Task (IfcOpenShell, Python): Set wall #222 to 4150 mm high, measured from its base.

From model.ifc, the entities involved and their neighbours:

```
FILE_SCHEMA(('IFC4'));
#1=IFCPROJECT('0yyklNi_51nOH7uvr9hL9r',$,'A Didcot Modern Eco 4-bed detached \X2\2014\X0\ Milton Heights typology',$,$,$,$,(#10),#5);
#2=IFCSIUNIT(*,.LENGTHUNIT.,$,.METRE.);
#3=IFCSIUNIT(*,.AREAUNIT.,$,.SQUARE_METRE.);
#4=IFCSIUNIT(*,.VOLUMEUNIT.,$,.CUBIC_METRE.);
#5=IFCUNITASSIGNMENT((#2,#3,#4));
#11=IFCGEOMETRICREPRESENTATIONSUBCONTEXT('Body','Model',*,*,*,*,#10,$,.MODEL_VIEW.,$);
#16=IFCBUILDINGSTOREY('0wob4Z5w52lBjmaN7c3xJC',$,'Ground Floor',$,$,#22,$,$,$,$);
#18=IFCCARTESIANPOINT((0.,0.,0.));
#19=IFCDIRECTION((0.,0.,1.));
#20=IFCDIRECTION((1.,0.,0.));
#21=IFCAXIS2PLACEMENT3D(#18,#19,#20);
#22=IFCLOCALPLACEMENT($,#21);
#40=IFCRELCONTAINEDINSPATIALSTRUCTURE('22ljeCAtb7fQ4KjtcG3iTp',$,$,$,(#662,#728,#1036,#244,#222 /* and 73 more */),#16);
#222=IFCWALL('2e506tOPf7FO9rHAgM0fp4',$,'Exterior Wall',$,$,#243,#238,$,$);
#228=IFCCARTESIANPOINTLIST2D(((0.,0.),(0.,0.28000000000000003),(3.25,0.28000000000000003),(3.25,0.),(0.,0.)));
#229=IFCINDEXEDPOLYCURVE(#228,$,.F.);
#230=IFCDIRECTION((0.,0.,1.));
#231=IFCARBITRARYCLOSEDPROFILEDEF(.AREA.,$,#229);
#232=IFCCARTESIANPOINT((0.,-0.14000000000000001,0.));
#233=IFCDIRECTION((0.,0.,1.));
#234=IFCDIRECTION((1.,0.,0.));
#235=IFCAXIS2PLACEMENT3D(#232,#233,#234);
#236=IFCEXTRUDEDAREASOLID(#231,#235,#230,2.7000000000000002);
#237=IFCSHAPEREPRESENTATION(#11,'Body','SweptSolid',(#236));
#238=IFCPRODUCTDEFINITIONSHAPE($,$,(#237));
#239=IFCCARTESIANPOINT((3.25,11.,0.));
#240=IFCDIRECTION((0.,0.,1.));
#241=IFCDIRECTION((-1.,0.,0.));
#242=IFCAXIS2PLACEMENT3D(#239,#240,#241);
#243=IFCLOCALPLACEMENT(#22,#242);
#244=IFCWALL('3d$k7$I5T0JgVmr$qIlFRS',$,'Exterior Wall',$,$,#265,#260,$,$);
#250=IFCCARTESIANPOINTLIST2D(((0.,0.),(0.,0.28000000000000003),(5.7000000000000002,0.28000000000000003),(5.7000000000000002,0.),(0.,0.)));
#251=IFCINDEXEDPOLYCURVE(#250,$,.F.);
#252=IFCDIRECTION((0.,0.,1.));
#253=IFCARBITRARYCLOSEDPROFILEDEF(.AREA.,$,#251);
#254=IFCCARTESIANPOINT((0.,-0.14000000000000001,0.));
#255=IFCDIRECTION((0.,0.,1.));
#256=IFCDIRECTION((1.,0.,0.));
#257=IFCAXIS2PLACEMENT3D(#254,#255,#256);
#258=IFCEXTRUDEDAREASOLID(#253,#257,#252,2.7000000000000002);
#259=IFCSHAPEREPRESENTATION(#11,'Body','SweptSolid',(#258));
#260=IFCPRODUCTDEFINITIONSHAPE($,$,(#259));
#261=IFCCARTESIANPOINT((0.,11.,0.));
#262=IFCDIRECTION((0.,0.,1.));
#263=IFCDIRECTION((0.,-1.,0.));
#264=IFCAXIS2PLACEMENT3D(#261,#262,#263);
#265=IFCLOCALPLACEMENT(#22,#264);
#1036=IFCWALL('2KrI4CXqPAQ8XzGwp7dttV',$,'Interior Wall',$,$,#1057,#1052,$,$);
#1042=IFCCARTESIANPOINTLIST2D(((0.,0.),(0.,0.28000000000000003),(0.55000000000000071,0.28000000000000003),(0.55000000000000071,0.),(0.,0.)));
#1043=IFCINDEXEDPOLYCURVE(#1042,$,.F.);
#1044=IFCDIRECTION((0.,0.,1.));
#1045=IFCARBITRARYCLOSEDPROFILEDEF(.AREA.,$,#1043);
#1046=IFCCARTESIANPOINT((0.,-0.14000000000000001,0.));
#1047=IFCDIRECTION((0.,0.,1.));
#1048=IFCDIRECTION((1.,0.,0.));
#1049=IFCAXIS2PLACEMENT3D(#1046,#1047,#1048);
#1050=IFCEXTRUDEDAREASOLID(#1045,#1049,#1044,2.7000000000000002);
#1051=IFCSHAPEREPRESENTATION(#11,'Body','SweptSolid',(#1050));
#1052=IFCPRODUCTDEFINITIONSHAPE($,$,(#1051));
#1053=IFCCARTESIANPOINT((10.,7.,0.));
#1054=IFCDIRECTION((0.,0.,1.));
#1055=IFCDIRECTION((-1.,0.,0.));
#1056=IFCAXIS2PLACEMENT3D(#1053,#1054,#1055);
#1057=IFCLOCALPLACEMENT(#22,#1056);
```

```python
import ifcopenshell
import ifcopenshell.geom
import ifcopenshell.util.representation
import ifcopenshell.util.shape
import ifcopenshell.util.unit

model = ifcopenshell.open("model.ifc")
unit_scale = ifcopenshell.util.unit.calculate_unit_scale(model)
settings = ifcopenshell.geom.settings()


def volume(element):
    """Net volume in cubic metres, openings subtracted."""
    shape = ifcopenshell.geom.create_shape(settings, element)
    return ifcopenshell.util.shape.get_volume(shape.geometry)


wall = model.by_id(222)
before = volume(wall)

body = ifcopenshell.util.representation.get_representation(wall, "Model", "Body")
solid = body.Items[0]
old_height = solid.Depth
solid.Depth = 4.15 / unit_scale
after = volume(wall)

print(f"height {old_height:g} -> {solid.Depth:g}, volume {before:.3f} -> {after:.3f} m3")

model.write("model_v2.ifc")
```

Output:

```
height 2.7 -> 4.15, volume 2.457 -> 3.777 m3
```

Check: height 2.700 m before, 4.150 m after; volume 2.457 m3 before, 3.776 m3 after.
